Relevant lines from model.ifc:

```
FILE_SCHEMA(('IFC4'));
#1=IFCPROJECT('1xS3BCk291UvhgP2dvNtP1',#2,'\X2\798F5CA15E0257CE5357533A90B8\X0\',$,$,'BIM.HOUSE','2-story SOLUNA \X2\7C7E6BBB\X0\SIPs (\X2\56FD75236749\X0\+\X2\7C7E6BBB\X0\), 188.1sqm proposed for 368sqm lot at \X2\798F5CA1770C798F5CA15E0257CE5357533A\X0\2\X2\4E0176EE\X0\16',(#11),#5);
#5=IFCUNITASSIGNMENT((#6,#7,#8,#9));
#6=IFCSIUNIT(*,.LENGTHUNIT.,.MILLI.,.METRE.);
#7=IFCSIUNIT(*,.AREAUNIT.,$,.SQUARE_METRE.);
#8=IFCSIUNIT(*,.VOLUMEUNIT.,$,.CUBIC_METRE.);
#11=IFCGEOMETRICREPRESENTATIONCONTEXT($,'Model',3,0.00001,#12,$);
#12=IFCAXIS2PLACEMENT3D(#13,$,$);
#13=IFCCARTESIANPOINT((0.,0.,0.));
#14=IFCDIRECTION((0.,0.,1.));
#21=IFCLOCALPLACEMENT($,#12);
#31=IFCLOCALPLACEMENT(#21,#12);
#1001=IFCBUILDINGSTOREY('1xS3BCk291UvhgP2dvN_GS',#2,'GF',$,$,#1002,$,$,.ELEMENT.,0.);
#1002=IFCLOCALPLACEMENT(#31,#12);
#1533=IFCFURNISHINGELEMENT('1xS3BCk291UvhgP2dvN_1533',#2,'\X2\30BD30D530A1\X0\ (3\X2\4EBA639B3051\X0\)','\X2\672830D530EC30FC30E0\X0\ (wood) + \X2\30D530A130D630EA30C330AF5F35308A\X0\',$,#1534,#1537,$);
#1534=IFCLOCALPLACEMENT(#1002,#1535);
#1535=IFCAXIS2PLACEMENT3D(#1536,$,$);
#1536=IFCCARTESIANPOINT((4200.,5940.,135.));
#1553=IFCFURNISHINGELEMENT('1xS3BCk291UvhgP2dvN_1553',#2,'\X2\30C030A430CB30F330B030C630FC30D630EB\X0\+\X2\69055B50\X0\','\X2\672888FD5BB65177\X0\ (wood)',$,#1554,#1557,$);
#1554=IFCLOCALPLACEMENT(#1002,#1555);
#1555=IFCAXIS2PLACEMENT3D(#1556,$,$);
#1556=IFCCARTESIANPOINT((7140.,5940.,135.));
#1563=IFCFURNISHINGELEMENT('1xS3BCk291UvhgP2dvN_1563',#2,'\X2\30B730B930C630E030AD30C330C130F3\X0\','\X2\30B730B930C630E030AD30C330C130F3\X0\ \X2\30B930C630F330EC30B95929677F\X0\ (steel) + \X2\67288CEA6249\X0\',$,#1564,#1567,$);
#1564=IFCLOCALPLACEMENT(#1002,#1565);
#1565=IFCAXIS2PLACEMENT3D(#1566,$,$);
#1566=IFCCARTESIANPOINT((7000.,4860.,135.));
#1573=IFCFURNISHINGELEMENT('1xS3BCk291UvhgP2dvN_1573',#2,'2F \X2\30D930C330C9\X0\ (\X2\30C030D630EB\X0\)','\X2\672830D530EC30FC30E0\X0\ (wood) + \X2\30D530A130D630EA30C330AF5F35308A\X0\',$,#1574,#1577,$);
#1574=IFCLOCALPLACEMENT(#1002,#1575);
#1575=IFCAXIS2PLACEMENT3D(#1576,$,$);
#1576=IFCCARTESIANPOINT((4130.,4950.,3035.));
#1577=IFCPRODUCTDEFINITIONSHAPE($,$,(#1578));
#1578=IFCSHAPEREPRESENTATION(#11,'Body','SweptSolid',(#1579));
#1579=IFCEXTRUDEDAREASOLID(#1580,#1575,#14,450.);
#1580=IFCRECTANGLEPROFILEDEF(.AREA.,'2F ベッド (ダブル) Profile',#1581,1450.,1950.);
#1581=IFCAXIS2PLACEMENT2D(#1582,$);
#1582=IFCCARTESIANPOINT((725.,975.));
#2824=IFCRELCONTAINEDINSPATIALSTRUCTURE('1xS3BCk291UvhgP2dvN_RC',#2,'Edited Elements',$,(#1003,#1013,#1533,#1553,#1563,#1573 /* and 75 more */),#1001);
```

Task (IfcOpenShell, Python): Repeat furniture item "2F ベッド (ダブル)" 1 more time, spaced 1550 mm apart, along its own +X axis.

```python
import ifcopenshell
import ifcopenshell.api.geometry
import ifcopenshell.api.root
import ifcopenshell.util.element
import ifcopenshell.util.placement
import ifcopenshell.util.unit

model = ifcopenshell.open("model.ifc")
unit_scale = ifcopenshell.util.unit.calculate_unit_scale(model)


def reuse_history(source, copy):
    """copy_class also copies each property set's owner history, people and application; keep the originals."""
    for rel in copy.IsDefinedBy:
        if rel.is_a("IfcRelDefinesByProperties") and (history := rel.RelatingPropertyDefinition.OwnerHistory):
            rel.RelatingPropertyDefinition.OwnerHistory = source.OwnerHistory
            ifcopenshell.util.element.remove_deep2(model, history)


source = model.by_guid("1xS3BCk291UvhgP2dvN_1573")
base = ifcopenshell.util.placement.get_local_placement(source.ObjectPlacement)
step = base[:3, 0] * 1.55 / unit_scale

for i in range(1, 2):
    copy = ifcopenshell.api.root.copy_class(model, product=source)
    copy.Representation = ifcopenshell.util.element.copy_deep(
        model, source.Representation, exclude=["IfcGeometricRepresentationContext", "IfcRepresentationMap"]
    )
    reuse_history(source, copy)
    matrix = base.copy()
    matrix[:3, 3] += i * step
    print("added at", matrix[:3, 3].round(3) + 0.0)
    ifcopenshell.api.geometry.edit_object_placement(model, product=copy, matrix=matrix, is_si=False)

model.write("model_edited.ifc")
```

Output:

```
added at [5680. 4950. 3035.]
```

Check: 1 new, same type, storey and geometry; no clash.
